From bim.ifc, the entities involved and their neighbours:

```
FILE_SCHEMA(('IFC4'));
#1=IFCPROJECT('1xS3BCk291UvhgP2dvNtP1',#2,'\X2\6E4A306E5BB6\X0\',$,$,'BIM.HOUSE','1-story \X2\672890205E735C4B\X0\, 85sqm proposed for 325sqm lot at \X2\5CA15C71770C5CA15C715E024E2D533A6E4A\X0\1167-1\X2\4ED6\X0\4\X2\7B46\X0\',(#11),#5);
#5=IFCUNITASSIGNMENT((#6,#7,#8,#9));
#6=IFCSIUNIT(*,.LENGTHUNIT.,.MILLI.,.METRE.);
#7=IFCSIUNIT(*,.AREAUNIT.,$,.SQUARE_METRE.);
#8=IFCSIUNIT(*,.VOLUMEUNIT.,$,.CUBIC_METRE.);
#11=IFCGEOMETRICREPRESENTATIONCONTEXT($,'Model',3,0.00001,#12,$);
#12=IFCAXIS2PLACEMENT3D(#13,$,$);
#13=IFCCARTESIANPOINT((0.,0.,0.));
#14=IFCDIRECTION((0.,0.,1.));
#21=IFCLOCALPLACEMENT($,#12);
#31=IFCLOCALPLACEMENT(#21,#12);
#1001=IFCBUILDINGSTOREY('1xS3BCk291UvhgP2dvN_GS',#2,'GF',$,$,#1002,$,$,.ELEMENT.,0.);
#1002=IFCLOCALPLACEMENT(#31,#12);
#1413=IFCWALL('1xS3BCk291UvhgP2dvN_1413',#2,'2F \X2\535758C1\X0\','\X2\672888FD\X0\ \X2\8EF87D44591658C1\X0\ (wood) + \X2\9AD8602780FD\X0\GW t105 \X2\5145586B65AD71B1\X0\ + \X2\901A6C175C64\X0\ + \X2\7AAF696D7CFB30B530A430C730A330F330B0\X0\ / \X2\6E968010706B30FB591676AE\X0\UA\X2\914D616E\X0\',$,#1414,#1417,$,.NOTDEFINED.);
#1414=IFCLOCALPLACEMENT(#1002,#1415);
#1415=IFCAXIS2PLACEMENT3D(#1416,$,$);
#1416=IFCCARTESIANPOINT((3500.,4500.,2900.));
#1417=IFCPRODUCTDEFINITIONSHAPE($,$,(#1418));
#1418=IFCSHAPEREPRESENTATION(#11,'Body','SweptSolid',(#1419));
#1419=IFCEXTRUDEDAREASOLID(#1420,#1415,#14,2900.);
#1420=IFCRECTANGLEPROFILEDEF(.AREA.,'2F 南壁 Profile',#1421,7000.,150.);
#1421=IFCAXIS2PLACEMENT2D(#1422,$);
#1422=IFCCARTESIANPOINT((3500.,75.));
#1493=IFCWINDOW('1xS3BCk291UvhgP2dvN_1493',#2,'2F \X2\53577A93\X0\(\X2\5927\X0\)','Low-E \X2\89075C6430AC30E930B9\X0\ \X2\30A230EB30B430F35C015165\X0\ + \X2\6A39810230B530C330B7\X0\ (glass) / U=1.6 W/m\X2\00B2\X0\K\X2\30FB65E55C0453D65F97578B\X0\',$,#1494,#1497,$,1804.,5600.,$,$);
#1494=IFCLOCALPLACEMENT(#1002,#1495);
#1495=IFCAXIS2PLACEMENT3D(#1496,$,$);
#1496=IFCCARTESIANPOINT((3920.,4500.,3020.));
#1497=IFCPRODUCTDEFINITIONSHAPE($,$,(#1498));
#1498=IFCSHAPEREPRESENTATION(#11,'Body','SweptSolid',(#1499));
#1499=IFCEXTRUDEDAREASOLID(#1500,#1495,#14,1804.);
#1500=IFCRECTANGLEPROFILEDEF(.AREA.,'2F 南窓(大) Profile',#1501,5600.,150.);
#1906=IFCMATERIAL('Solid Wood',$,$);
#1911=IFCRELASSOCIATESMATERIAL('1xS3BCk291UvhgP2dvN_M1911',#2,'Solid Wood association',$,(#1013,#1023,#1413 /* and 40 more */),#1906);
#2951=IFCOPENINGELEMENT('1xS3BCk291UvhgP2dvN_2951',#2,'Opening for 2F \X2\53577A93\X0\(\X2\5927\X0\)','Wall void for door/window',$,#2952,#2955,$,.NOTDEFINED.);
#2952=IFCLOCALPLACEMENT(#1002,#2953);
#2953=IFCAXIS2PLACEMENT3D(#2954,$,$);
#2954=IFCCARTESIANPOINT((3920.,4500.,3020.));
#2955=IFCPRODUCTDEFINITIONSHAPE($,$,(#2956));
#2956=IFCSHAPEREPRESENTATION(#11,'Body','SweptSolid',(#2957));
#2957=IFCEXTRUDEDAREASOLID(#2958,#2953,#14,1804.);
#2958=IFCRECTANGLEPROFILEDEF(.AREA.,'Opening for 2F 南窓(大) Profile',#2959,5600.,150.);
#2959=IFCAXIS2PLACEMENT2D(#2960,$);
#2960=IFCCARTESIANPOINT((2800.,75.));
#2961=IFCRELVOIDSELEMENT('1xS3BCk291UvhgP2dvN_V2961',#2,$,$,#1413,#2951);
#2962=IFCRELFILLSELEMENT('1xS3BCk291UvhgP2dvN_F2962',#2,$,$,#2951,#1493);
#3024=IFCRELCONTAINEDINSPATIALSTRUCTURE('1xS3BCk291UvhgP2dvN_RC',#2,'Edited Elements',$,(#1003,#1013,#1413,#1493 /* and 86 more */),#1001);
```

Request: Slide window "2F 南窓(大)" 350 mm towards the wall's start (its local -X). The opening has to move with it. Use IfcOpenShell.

```python
import ifcopenshell
import ifcopenshell.api.geometry
import ifcopenshell.util.placement
import ifcopenshell.util.unit

model = ifcopenshell.open("bim.ifc")
unit_scale = ifcopenshell.util.unit.calculate_unit_scale(model)

window = model.by_guid("1xS3BCk291UvhgP2dvN_1493")
opening = window.FillsVoids[0].RelatingOpeningElement
wall = opening.VoidsElements[0].RelatingBuildingElement

wall_matrix = ifcopenshell.util.placement.get_local_placement(wall.ObjectPlacement)
shift = wall_matrix[:3, 0] * -0.35 / unit_scale
before = ifcopenshell.util.placement.get_local_placement(window.ObjectPlacement)[:3, 3].copy()

# The window is not placed relative to its opening, so move both.
for product in (opening, window):
    matrix = ifcopenshell.util.placement.get_local_placement(product.ObjectPlacement)
    matrix[:3, 3] += shift
    ifcopenshell.api.geometry.edit_object_placement(model, product=product, matrix=matrix, is_si=False)

after = ifcopenshell.util.placement.get_local_placement(window.ObjectPlacement)[:3, 3]
print("window moved by", (after - before).round(3) + 0.0)

model.write("bim_rev.ifc")
```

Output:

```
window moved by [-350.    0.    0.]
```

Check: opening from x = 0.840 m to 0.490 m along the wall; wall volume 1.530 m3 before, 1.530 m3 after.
